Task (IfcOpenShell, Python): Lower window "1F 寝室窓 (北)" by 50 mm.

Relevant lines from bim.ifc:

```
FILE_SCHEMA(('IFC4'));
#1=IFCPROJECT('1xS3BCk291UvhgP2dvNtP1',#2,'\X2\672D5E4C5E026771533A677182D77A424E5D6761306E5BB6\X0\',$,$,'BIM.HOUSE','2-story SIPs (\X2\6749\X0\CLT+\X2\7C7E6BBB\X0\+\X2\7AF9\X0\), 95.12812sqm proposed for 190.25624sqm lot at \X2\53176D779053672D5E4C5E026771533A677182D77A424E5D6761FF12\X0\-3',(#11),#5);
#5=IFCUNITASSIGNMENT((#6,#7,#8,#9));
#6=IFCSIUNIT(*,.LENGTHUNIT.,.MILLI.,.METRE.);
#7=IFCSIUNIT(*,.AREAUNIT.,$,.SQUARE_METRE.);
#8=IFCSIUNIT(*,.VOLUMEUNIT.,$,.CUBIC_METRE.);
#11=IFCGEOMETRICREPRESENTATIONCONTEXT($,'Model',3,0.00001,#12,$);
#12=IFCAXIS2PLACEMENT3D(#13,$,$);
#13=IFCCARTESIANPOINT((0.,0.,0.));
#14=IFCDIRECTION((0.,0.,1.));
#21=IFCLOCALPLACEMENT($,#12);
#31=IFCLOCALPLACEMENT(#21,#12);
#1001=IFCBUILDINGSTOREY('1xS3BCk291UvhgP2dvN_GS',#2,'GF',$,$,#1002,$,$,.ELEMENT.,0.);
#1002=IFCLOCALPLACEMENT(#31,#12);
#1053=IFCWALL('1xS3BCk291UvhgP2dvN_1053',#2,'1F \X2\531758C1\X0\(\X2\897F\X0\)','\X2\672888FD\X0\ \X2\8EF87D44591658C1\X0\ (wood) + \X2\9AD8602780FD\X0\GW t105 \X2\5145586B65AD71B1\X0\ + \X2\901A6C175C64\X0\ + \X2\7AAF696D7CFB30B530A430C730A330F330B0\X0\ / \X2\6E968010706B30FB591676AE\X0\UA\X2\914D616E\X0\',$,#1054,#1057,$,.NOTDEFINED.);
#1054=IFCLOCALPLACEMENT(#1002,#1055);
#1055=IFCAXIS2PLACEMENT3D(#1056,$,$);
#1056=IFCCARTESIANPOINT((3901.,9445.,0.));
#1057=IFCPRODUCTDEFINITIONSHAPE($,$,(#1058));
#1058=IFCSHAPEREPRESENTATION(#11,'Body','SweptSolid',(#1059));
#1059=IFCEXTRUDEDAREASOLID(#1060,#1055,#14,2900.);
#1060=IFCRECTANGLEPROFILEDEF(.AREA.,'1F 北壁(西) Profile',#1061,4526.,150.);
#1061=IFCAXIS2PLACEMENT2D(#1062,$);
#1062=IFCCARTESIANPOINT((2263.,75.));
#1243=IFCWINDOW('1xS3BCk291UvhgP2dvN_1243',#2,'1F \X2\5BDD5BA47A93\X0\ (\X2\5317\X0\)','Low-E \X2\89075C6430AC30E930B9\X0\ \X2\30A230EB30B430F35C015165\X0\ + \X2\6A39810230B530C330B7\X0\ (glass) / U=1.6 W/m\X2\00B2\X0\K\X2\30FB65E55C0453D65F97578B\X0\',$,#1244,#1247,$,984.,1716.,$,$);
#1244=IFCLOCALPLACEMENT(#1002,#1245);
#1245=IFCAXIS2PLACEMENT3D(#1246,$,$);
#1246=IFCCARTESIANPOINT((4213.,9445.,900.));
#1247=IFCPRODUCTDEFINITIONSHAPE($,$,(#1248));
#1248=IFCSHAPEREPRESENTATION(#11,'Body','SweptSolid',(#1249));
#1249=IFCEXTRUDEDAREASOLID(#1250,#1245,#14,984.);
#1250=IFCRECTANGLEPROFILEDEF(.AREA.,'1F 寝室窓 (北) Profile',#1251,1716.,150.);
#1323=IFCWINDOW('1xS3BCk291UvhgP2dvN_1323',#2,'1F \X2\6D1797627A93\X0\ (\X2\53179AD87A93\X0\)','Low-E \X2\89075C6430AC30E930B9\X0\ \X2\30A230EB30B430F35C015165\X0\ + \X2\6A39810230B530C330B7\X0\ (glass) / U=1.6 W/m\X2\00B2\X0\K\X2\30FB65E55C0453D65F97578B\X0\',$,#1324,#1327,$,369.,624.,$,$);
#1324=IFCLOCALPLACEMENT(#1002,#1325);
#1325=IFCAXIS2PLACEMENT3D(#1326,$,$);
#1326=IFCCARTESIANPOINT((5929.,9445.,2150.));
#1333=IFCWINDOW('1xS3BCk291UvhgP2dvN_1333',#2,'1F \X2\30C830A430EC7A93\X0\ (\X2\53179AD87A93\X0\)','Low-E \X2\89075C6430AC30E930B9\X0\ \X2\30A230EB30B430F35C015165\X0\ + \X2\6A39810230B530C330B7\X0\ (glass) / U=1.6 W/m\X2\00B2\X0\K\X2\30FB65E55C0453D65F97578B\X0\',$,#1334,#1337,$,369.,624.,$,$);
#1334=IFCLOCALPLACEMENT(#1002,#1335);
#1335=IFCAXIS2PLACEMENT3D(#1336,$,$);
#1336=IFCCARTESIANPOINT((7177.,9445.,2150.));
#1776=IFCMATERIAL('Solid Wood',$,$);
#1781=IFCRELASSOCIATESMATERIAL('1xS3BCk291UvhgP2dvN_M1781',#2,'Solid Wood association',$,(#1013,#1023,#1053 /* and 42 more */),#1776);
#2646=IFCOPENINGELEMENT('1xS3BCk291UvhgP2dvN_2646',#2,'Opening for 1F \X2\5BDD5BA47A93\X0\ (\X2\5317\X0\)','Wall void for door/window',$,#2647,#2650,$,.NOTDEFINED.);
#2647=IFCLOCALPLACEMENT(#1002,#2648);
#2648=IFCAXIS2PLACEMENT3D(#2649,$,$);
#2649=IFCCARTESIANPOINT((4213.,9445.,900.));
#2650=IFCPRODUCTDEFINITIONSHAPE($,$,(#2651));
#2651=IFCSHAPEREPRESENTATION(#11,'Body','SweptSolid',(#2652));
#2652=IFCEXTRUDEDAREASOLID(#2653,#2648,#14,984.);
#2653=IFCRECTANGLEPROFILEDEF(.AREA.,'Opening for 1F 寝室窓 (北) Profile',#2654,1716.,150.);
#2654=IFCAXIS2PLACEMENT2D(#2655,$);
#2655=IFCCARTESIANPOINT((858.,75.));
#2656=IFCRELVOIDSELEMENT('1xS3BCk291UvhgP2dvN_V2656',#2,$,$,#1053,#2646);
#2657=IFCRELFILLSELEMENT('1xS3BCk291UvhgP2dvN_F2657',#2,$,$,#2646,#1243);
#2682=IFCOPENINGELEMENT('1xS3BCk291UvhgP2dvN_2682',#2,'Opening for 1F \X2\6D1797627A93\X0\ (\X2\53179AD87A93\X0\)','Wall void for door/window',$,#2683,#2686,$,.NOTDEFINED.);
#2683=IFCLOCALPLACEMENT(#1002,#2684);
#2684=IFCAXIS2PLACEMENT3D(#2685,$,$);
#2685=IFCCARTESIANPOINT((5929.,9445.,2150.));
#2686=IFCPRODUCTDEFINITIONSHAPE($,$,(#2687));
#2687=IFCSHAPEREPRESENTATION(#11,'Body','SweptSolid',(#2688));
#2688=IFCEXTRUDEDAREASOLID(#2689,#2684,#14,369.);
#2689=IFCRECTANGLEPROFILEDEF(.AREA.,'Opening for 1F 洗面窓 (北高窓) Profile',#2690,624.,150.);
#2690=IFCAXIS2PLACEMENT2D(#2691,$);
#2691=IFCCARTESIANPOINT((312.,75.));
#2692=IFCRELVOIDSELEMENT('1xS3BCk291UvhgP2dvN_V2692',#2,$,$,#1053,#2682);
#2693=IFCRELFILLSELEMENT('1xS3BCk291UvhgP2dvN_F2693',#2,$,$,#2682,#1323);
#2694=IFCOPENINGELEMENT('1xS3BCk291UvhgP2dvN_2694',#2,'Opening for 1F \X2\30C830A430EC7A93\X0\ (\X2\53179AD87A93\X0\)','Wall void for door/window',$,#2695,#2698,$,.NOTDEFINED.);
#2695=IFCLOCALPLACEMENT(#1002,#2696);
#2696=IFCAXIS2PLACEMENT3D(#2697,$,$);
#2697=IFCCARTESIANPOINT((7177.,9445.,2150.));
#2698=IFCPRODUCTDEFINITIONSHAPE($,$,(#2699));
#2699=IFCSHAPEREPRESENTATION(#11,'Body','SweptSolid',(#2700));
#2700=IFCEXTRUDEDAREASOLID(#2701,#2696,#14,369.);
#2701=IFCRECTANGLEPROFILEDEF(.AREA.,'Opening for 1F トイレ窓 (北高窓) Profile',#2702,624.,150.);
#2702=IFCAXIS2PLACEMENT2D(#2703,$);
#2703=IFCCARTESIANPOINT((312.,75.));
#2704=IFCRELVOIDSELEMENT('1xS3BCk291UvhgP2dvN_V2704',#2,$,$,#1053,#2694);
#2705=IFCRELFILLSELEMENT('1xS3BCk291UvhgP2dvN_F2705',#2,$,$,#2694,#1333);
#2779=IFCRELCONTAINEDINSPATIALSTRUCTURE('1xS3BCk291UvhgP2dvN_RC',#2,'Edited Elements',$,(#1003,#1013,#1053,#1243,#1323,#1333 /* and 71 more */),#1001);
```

```python
import numpy as np
import ifcopenshell
import ifcopenshell.api.geometry
import ifcopenshell.util.placement
import ifcopenshell.util.unit

model = ifcopenshell.open("bim.ifc")
unit_scale = ifcopenshell.util.unit.calculate_unit_scale(model)

window = model.by_guid("1xS3BCk291UvhgP2dvN_1243")
opening = window.FillsVoids[0].RelatingOpeningElement
dz = -50.0

shift = np.array([0.0, 0.0, dz])
# The window is not placed relative to its opening, so move both.
for product in (opening, window):
    matrix = ifcopenshell.util.placement.get_local_placement(product.ObjectPlacement)
    matrix[:3, 3] += shift
    ifcopenshell.api.geometry.edit_object_placement(model, product=product, matrix=matrix, is_si=False)

print(f"moved by {dz * unit_scale:+.3f} m")

model.write("bim_updated.ifc")
```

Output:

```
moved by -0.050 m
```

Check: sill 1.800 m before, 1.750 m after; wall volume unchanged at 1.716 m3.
